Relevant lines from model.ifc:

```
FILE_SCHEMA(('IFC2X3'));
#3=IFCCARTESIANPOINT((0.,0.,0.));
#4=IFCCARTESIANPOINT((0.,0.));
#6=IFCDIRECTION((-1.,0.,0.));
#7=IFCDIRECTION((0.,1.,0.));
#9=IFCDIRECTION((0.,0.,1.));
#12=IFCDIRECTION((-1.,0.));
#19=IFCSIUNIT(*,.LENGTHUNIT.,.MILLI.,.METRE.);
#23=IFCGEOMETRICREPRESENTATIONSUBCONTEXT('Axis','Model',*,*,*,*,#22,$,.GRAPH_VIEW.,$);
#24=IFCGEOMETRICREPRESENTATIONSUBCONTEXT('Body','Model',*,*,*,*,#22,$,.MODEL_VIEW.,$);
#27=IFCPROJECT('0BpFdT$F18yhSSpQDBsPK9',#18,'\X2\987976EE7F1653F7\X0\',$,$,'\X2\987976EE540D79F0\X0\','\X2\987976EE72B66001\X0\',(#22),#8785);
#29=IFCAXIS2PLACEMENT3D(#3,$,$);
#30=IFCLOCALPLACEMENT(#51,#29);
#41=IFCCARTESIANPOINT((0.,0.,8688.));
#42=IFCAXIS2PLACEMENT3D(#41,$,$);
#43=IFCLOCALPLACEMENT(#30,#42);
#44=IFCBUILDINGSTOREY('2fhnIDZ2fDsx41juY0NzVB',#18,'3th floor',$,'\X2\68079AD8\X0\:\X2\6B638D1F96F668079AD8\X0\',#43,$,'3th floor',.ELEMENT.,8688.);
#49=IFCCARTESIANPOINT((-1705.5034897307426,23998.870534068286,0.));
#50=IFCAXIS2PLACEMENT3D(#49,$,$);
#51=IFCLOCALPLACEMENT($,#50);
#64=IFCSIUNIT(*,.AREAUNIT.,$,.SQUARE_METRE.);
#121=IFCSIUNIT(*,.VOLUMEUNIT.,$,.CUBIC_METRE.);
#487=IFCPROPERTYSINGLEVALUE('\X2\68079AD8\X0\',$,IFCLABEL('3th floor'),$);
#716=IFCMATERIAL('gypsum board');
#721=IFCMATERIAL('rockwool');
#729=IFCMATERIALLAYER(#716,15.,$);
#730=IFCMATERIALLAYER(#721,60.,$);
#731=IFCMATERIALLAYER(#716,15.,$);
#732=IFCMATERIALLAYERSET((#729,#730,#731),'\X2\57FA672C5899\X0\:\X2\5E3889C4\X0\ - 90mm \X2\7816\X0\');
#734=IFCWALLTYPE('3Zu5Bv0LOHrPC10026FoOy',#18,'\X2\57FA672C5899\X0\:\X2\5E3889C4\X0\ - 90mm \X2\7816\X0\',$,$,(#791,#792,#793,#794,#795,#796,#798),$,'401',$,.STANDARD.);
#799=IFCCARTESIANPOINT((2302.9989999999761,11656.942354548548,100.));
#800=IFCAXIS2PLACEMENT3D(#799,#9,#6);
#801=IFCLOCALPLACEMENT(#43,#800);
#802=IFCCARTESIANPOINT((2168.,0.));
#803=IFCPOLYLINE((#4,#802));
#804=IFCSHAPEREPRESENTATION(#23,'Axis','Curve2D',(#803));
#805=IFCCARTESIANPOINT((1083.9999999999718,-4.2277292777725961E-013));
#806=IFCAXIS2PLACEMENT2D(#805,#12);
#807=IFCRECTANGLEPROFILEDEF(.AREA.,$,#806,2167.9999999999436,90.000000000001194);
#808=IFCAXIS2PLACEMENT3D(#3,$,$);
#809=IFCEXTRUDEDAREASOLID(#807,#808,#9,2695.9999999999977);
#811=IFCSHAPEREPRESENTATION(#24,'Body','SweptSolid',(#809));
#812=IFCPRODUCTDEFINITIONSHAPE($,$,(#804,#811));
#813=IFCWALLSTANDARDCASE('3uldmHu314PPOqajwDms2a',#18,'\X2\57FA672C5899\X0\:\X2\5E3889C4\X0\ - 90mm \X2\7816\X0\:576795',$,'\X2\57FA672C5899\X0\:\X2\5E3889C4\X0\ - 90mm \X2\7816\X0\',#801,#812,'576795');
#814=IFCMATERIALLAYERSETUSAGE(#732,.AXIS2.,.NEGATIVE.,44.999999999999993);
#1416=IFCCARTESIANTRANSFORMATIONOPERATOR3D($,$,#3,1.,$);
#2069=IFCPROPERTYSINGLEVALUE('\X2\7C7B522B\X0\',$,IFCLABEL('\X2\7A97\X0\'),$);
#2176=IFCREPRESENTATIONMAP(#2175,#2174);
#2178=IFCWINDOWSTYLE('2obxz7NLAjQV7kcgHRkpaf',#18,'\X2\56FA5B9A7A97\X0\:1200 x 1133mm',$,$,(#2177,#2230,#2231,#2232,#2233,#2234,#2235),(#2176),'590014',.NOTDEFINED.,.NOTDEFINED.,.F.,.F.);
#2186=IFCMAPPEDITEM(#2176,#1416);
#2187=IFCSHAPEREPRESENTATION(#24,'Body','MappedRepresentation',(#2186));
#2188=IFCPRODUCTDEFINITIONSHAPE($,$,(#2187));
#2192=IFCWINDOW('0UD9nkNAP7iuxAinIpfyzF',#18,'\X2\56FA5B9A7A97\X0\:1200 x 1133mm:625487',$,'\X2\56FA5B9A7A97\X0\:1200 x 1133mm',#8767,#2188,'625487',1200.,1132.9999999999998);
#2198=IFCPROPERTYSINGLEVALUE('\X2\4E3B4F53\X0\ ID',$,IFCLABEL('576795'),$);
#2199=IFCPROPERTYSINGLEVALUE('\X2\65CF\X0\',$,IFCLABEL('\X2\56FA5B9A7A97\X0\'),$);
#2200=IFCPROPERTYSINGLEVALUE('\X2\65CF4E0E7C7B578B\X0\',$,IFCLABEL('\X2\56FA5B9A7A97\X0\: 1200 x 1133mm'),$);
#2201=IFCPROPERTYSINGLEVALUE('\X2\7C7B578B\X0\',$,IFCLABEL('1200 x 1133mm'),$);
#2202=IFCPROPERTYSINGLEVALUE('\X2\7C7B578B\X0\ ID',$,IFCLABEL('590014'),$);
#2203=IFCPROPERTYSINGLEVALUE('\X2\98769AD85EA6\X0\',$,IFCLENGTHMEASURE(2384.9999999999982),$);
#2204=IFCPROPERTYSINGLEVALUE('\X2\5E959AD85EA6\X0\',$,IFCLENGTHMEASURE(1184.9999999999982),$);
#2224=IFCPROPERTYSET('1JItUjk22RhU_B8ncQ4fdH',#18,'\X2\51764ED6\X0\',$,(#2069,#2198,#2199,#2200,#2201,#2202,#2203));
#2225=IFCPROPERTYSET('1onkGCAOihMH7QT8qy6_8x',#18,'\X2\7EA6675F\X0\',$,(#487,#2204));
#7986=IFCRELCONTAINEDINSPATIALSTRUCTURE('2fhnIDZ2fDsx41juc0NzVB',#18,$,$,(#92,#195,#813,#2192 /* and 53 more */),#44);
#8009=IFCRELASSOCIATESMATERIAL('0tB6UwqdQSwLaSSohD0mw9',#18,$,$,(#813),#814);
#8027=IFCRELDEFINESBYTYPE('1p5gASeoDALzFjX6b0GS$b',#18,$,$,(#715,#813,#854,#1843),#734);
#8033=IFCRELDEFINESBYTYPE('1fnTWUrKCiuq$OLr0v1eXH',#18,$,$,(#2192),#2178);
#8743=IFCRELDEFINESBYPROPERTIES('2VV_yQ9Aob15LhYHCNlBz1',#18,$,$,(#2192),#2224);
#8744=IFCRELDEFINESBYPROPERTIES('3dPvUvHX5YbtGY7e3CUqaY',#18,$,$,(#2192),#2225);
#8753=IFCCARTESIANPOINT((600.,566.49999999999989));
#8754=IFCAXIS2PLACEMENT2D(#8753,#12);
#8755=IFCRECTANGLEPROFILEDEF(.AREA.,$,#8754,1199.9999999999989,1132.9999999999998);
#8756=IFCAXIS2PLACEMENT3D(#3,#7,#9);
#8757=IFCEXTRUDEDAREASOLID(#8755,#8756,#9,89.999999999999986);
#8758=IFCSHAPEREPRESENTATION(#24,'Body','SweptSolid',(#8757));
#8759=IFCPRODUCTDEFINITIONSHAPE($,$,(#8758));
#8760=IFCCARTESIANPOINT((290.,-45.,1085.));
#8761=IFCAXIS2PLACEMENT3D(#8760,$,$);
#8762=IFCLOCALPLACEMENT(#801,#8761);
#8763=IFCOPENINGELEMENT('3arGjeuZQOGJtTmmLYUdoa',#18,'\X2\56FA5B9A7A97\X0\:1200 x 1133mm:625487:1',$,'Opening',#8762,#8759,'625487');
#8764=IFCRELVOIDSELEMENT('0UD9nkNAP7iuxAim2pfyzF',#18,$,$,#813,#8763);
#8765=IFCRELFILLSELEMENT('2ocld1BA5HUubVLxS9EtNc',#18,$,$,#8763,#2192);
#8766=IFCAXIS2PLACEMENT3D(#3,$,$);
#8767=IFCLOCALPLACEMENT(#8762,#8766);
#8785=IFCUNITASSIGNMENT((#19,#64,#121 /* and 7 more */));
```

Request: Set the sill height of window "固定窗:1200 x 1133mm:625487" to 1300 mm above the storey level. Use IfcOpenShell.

```python
import numpy as np
import ifcopenshell
import ifcopenshell.api.geometry
import ifcopenshell.api.pset
import ifcopenshell.geom
import ifcopenshell.util.element
import ifcopenshell.util.placement
import ifcopenshell.util.shape
import ifcopenshell.util.unit

model = ifcopenshell.open("model.ifc")
unit_scale = ifcopenshell.util.unit.calculate_unit_scale(model)

window = model.by_guid("0UD9nkNAP7iuxAinIpfyzF")
opening = window.FillsVoids[0].RelatingOpeningElement
storey = ifcopenshell.util.element.get_container(window, ifc_class="IfcBuildingStorey")
level = ifcopenshell.util.placement.get_local_placement(storey.ObjectPlacement)[2, 3]

# The opening's origin need not be at the sill, so measure its lowest point.
shape = ifcopenshell.geom.create_shape(ifcopenshell.geom.settings(), opening)
bottom = ifcopenshell.util.shape.get_shape_bottom_elevation(shape, shape.geometry) / unit_scale
dz = level + 1300.0 - bottom

shift = np.array([0.0, 0.0, dz])
# The window is placed relative to its opening, so it follows when the opening moves.
matrix = ifcopenshell.util.placement.get_local_placement(opening.ObjectPlacement)
matrix[:3, 3] += shift
ifcopenshell.api.geometry.edit_object_placement(
    model, product=opening, matrix=matrix, is_si=False, should_transform_children=True
)

# Keep the stored heights in step.
pset = model.by_id(ifcopenshell.util.element.get_pset(window, "其他", should_inherit=False)["id"])
ifcopenshell.api.pset.edit_pset(model, pset=pset, properties={
    "顶高度": model.create_entity("IfcLengthMeasure", ifcopenshell.util.element.get_pset(window, "其他", "顶高度") + dz),
})
pset = model.by_id(ifcopenshell.util.element.get_pset(window, "约束", should_inherit=False)["id"])
ifcopenshell.api.pset.edit_pset(model, pset=pset, properties={
    "底高度": model.create_entity("IfcLengthMeasure", ifcopenshell.util.element.get_pset(window, "约束", "底高度") + dz),
})

print(f"moved by {dz * unit_scale:+.3f} m")

model.write("model_edited.ifc")
```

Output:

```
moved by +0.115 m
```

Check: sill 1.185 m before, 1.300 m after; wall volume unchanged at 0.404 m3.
